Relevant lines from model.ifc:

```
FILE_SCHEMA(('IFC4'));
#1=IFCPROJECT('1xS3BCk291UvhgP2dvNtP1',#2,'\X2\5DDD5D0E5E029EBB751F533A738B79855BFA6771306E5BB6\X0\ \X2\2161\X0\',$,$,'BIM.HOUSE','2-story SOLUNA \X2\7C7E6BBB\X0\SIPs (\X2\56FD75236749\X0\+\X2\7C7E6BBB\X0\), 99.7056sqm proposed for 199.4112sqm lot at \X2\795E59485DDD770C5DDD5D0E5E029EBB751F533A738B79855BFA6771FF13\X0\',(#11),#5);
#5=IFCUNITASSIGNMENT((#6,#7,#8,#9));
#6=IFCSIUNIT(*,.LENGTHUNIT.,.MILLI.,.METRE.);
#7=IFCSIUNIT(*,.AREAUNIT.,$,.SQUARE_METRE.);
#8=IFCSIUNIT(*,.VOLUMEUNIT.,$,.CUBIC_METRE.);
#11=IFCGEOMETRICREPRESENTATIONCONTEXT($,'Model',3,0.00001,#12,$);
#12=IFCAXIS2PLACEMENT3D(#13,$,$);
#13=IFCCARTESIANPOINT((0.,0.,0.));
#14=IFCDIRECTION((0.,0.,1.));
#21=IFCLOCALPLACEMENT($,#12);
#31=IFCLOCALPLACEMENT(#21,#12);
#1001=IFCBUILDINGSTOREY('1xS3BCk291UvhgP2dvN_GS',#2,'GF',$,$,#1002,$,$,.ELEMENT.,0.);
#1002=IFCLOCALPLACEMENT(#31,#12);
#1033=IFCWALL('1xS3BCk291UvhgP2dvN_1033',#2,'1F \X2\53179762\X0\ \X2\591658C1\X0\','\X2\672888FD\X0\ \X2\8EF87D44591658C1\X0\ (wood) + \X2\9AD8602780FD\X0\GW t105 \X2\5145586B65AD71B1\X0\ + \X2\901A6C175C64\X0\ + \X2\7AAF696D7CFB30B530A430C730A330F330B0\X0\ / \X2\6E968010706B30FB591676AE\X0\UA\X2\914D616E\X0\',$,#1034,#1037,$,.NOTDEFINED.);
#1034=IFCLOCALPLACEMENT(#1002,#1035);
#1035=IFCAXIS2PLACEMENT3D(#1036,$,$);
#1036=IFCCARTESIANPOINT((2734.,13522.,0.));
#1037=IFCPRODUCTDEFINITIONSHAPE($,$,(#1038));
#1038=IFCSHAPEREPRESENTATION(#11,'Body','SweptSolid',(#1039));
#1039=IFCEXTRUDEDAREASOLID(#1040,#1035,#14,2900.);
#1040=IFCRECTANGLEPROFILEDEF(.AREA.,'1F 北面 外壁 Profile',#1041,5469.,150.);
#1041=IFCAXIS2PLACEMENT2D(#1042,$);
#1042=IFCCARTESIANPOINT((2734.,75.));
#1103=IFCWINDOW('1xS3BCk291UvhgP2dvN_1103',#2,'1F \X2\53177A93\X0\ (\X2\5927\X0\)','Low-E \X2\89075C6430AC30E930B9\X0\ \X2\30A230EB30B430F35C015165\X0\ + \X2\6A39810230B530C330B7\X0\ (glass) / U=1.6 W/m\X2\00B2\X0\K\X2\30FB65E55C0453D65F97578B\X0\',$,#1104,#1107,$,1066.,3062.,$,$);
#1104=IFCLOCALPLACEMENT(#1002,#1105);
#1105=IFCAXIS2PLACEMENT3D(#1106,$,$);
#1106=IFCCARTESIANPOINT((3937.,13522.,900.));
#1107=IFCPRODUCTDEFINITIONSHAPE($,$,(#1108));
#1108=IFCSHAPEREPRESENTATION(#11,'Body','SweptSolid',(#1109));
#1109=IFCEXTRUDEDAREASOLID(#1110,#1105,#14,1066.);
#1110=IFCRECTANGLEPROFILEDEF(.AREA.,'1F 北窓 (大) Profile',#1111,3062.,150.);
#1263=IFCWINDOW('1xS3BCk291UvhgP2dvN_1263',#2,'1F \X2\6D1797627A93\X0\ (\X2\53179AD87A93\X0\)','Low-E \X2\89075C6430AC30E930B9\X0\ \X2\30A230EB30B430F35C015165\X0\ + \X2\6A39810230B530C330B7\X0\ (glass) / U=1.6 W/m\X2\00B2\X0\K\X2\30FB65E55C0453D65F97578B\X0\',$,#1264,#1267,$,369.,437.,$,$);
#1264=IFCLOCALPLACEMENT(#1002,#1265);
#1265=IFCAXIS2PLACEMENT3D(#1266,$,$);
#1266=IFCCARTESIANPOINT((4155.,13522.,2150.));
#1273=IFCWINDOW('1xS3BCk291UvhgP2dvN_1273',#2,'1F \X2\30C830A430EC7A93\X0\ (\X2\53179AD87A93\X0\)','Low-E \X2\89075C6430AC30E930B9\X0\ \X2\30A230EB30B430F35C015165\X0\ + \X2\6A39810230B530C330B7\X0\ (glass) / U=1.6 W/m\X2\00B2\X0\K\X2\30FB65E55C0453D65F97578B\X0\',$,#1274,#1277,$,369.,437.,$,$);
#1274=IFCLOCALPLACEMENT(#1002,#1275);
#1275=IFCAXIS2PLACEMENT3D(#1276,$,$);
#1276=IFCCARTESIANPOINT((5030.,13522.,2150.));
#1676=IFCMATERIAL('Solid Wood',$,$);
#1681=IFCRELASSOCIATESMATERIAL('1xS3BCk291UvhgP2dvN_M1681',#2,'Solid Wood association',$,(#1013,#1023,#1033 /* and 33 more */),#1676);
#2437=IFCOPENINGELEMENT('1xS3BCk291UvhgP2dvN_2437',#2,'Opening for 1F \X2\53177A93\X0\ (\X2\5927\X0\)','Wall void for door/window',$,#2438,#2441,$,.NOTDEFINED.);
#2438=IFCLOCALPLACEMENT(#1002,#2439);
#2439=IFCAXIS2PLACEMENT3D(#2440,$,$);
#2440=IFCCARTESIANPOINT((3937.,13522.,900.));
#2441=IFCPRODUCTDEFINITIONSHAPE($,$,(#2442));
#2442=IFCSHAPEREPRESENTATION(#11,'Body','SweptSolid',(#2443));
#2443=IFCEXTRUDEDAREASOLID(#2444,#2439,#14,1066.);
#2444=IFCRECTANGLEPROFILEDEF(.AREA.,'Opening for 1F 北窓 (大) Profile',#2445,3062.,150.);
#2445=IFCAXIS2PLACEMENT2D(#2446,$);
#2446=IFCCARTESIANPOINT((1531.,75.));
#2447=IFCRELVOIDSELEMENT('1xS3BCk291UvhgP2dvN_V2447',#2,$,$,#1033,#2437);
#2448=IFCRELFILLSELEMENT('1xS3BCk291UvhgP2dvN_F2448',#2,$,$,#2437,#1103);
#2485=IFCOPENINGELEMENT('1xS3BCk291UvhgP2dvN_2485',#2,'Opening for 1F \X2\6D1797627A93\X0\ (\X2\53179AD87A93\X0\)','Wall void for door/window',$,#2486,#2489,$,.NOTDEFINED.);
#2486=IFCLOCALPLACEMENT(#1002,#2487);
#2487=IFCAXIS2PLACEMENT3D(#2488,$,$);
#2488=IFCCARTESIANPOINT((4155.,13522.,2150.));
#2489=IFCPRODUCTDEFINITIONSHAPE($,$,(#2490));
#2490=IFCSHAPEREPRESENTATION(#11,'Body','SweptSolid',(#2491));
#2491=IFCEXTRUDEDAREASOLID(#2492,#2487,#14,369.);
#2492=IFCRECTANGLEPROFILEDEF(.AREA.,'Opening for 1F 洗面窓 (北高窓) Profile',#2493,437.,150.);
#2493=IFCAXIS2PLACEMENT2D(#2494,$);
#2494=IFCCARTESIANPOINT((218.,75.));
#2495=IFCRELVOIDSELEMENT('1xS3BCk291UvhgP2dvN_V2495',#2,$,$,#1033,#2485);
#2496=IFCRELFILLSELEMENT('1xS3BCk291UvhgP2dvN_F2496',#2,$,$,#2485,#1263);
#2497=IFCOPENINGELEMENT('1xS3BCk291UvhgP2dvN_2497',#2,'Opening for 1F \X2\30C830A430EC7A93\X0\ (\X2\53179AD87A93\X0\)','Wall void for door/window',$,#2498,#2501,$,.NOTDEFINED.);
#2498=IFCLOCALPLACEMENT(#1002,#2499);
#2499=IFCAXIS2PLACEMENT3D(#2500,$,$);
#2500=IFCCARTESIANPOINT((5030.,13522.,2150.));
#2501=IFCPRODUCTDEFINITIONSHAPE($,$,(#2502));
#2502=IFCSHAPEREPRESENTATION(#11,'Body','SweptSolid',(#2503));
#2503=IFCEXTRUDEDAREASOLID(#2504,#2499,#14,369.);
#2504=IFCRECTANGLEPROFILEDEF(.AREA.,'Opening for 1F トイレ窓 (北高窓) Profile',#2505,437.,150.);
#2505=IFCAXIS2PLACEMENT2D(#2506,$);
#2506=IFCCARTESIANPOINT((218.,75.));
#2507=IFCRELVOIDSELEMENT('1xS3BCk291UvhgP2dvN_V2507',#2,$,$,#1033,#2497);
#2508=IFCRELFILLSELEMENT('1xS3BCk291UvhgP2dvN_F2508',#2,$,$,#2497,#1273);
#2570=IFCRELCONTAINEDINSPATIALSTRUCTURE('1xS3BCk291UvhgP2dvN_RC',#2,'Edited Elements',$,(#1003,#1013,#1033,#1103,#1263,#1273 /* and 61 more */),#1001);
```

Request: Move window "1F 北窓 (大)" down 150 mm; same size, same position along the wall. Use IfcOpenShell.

```python
import numpy as np
import ifcopenshell
import ifcopenshell.api.geometry
import ifcopenshell.util.placement
import ifcopenshell.util.unit

model = ifcopenshell.open("model.ifc")
unit_scale = ifcopenshell.util.unit.calculate_unit_scale(model)

window = model.by_guid("1xS3BCk291UvhgP2dvN_1103")
opening = window.FillsVoids[0].RelatingOpeningElement
dz = -0.15 / unit_scale

shift = np.array([0.0, 0.0, dz])
# The window is not placed relative to its opening, so move both.
for product in (opening, window):
    matrix = ifcopenshell.util.placement.get_local_placement(product.ObjectPlacement)
    matrix[:3, 3] += shift
    ifcopenshell.api.geometry.edit_object_placement(model, product=product, matrix=matrix, is_si=False)

print(f"moved by {dz * unit_scale:+.3f} m")

model.write("model_updated.ifc")
```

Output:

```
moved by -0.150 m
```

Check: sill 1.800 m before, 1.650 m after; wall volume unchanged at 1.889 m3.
